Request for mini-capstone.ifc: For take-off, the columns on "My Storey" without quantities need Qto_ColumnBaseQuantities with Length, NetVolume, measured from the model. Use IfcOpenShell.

First a look at what the model holds.

```python
import ifcopenshell
import ifcopenshell.util.element
import ifcopenshell.util.unit

model = ifcopenshell.open("mini-capstone.ifc")
print(model.schema)
for unit_type in ("LENGTHUNIT", "AREAUNIT", "VOLUMEUNIT"):
    print(unit_type, ifcopenshell.util.unit.calculate_unit_scale(model, unit_type))
storey = next(s for s in model.by_type("IfcBuildingStorey") if s.Name == "My Storey")
columns = [e for e in ifcopenshell.util.element.get_decomposition(storey) if e.is_a("IfcColumn")]
for e in sorted(columns, key=lambda e: e.id()):
    print(e.id(), e.is_a(), e.Name, list(ifcopenshell.util.element.get_psets(e, qtos_only=True)), sep=" | ")
```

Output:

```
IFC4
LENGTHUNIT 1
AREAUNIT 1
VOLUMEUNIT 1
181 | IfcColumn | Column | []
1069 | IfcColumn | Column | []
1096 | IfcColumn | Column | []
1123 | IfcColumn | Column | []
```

```python
import ifcopenshell
import ifcopenshell.api.pset
import ifcopenshell.geom
import ifcopenshell.util.element
import ifcopenshell.util.shape
import ifcopenshell.util.unit

model = ifcopenshell.open("mini-capstone.ifc")
unit_scale = ifcopenshell.util.unit.calculate_unit_scale(model)
volume_scale = ifcopenshell.util.unit.calculate_unit_scale(model, "VOLUMEUNIT")
settings = ifcopenshell.geom.settings()

storey = next(s for s in model.by_type("IfcBuildingStorey") if s.Name == "My Storey")
columns = [e for e in ifcopenshell.util.element.get_decomposition(storey) if e.is_a("IfcColumn")]

for e in sorted(columns, key=lambda e: e.id()):
    if ifcopenshell.util.element.get_psets(e, qtos_only=True, should_inherit=False):
        continue
    # Geometry comes back in metres, in the element's own axes.
    shape = ifcopenshell.geom.create_shape(settings, e)
    values = {
        "Length": ifcopenshell.util.shape.get_z(shape.geometry) / unit_scale,
        "NetVolume": ifcopenshell.util.shape.get_volume(shape.geometry) / volume_scale,
    }
    qto = ifcopenshell.api.pset.add_qto(model, product=e, name="Qto_ColumnBaseQuantities")
    ifcopenshell.api.pset.edit_qto(model, qto=qto, properties=values)
    print(e.id(), {k: round(v, 3) for k, v in values.items()})

model.write("mini-capstone_updated.ifc")
```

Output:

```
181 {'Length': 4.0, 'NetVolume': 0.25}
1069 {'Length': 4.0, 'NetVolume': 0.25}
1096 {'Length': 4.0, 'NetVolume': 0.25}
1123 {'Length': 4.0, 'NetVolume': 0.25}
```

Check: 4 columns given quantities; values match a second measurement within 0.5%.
